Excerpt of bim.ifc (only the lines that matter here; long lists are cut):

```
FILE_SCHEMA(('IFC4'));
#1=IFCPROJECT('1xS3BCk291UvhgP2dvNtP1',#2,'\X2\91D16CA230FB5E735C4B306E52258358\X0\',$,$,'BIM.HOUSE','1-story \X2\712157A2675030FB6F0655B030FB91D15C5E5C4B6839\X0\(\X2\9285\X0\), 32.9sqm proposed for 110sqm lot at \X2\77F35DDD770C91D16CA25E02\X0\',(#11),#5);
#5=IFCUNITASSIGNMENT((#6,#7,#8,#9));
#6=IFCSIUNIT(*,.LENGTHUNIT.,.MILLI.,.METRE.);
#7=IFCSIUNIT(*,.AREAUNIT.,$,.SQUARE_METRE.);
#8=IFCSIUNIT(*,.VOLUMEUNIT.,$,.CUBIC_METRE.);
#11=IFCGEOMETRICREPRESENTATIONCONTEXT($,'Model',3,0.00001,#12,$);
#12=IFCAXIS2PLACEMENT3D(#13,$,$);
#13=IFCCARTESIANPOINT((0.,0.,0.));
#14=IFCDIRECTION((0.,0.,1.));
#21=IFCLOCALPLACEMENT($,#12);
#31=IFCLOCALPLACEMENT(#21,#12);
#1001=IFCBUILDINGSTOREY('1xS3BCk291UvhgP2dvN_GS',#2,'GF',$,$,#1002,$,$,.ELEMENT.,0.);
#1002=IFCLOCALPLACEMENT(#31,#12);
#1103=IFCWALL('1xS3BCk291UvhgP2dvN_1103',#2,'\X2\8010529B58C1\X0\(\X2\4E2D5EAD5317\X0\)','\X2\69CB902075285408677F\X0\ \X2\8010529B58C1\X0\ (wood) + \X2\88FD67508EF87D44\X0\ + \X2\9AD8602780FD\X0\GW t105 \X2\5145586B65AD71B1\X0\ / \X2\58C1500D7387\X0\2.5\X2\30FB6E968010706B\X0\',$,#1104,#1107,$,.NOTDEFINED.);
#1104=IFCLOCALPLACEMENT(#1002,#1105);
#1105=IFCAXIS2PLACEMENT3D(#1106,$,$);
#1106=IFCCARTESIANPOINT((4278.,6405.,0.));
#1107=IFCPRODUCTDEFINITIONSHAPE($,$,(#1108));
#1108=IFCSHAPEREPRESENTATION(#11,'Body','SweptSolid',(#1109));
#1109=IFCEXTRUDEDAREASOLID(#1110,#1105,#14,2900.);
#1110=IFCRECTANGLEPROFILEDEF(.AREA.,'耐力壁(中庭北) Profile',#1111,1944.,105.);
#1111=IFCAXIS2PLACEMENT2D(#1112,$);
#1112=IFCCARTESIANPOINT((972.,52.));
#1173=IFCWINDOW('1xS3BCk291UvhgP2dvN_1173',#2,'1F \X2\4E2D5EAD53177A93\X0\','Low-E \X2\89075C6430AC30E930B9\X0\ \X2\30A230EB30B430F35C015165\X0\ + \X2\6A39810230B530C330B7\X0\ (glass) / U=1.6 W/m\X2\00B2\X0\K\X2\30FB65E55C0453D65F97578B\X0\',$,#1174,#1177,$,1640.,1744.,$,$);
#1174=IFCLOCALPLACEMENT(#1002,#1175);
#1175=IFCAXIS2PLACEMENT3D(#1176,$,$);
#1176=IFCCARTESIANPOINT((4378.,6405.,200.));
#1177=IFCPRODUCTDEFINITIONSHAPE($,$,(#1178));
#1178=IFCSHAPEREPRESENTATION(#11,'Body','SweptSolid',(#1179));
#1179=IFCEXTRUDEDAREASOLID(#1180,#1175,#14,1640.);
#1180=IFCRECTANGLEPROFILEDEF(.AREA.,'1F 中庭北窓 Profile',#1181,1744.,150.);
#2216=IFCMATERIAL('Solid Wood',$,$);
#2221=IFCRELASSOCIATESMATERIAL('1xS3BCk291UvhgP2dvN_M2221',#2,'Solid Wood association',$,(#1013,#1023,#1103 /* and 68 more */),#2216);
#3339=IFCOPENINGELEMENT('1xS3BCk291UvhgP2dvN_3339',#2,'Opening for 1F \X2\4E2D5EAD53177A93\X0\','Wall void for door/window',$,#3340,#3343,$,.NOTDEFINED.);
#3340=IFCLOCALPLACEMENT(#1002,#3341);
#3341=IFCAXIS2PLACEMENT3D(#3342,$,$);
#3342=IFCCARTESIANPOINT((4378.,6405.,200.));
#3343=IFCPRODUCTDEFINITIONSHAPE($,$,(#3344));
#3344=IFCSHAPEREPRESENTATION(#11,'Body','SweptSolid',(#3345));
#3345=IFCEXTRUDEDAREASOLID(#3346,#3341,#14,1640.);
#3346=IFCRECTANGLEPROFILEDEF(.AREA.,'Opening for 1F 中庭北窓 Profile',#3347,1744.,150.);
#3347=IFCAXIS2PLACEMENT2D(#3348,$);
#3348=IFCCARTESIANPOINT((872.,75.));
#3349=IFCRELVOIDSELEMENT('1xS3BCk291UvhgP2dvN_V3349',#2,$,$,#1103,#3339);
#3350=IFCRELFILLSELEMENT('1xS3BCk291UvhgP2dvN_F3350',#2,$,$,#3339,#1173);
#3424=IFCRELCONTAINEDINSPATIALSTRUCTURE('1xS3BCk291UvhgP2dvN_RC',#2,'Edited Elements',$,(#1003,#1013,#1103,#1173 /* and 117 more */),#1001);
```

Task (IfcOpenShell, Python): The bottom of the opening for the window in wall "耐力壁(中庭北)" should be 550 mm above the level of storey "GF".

```python
import numpy as np
import ifcopenshell
import ifcopenshell.api.geometry
import ifcopenshell.geom
import ifcopenshell.util.element
import ifcopenshell.util.placement
import ifcopenshell.util.shape
import ifcopenshell.util.unit

model = ifcopenshell.open("bim.ifc")
unit_scale = ifcopenshell.util.unit.calculate_unit_scale(model)

window = model.by_guid("1xS3BCk291UvhgP2dvN_1173")
opening = window.FillsVoids[0].RelatingOpeningElement
storey = ifcopenshell.util.element.get_container(window, ifc_class="IfcBuildingStorey")
level = ifcopenshell.util.placement.get_local_placement(storey.ObjectPlacement)[2, 3]

# The opening's origin need not be at the sill, so measure its lowest point.
shape = ifcopenshell.geom.create_shape(ifcopenshell.geom.settings(), opening)
bottom = ifcopenshell.util.shape.get_shape_bottom_elevation(shape, shape.geometry) / unit_scale
dz = level + 0.55 / unit_scale - bottom

shift = np.array([0.0, 0.0, dz])
# The window is not placed relative to its opening, so move both.
for product in (opening, window):
    matrix = ifcopenshell.util.placement.get_local_placement(product.ObjectPlacement)
    matrix[:3, 3] += shift
    ifcopenshell.api.geometry.edit_object_placement(model, product=product, matrix=matrix, is_si=False)

print(f"moved by {dz * unit_scale:+.3f} m")

model.write("bim_edited.ifc")
```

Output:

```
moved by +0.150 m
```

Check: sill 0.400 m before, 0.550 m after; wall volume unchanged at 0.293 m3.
